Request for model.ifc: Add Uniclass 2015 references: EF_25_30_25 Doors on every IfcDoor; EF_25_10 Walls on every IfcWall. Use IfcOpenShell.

First a look at what the model holds.

```python
import ifcopenshell

model = ifcopenshell.open("model.ifc")
print(model.schema)
print("classifications:", [c.Name for c in model.by_type("IfcClassification")])
for ifc_class in ("IfcDoor", "IfcRoof", "IfcStair", "IfcWall", "IfcWindow"):
    print(ifc_class, len(model.by_type(ifc_class)))
```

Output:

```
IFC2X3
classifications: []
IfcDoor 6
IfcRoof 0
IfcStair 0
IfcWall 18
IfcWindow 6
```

```python
import ifcopenshell
import ifcopenshell.api.classification

model = ifcopenshell.open("model.ifc")

# IFC2X3 requires Source and Edition and has no link from the project to the system.
system = model.create_entity("IfcClassification", Source="NBS", Edition="2015", Name="Uniclass 2015")

codes = {
    "IfcDoor": ("EF_25_30_25", "Doors"),
    "IfcWall": ("EF_25_10", "Walls"),
}
for ifc_class, (code, name) in codes.items():
    products = model.by_type(ifc_class)
    ifcopenshell.api.classification.add_reference(
        model, products=products, classification=system, identification=code, name=name
    )
    print(code, len(products))

model.write("model_edited.ifc")
```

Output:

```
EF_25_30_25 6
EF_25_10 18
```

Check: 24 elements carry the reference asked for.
